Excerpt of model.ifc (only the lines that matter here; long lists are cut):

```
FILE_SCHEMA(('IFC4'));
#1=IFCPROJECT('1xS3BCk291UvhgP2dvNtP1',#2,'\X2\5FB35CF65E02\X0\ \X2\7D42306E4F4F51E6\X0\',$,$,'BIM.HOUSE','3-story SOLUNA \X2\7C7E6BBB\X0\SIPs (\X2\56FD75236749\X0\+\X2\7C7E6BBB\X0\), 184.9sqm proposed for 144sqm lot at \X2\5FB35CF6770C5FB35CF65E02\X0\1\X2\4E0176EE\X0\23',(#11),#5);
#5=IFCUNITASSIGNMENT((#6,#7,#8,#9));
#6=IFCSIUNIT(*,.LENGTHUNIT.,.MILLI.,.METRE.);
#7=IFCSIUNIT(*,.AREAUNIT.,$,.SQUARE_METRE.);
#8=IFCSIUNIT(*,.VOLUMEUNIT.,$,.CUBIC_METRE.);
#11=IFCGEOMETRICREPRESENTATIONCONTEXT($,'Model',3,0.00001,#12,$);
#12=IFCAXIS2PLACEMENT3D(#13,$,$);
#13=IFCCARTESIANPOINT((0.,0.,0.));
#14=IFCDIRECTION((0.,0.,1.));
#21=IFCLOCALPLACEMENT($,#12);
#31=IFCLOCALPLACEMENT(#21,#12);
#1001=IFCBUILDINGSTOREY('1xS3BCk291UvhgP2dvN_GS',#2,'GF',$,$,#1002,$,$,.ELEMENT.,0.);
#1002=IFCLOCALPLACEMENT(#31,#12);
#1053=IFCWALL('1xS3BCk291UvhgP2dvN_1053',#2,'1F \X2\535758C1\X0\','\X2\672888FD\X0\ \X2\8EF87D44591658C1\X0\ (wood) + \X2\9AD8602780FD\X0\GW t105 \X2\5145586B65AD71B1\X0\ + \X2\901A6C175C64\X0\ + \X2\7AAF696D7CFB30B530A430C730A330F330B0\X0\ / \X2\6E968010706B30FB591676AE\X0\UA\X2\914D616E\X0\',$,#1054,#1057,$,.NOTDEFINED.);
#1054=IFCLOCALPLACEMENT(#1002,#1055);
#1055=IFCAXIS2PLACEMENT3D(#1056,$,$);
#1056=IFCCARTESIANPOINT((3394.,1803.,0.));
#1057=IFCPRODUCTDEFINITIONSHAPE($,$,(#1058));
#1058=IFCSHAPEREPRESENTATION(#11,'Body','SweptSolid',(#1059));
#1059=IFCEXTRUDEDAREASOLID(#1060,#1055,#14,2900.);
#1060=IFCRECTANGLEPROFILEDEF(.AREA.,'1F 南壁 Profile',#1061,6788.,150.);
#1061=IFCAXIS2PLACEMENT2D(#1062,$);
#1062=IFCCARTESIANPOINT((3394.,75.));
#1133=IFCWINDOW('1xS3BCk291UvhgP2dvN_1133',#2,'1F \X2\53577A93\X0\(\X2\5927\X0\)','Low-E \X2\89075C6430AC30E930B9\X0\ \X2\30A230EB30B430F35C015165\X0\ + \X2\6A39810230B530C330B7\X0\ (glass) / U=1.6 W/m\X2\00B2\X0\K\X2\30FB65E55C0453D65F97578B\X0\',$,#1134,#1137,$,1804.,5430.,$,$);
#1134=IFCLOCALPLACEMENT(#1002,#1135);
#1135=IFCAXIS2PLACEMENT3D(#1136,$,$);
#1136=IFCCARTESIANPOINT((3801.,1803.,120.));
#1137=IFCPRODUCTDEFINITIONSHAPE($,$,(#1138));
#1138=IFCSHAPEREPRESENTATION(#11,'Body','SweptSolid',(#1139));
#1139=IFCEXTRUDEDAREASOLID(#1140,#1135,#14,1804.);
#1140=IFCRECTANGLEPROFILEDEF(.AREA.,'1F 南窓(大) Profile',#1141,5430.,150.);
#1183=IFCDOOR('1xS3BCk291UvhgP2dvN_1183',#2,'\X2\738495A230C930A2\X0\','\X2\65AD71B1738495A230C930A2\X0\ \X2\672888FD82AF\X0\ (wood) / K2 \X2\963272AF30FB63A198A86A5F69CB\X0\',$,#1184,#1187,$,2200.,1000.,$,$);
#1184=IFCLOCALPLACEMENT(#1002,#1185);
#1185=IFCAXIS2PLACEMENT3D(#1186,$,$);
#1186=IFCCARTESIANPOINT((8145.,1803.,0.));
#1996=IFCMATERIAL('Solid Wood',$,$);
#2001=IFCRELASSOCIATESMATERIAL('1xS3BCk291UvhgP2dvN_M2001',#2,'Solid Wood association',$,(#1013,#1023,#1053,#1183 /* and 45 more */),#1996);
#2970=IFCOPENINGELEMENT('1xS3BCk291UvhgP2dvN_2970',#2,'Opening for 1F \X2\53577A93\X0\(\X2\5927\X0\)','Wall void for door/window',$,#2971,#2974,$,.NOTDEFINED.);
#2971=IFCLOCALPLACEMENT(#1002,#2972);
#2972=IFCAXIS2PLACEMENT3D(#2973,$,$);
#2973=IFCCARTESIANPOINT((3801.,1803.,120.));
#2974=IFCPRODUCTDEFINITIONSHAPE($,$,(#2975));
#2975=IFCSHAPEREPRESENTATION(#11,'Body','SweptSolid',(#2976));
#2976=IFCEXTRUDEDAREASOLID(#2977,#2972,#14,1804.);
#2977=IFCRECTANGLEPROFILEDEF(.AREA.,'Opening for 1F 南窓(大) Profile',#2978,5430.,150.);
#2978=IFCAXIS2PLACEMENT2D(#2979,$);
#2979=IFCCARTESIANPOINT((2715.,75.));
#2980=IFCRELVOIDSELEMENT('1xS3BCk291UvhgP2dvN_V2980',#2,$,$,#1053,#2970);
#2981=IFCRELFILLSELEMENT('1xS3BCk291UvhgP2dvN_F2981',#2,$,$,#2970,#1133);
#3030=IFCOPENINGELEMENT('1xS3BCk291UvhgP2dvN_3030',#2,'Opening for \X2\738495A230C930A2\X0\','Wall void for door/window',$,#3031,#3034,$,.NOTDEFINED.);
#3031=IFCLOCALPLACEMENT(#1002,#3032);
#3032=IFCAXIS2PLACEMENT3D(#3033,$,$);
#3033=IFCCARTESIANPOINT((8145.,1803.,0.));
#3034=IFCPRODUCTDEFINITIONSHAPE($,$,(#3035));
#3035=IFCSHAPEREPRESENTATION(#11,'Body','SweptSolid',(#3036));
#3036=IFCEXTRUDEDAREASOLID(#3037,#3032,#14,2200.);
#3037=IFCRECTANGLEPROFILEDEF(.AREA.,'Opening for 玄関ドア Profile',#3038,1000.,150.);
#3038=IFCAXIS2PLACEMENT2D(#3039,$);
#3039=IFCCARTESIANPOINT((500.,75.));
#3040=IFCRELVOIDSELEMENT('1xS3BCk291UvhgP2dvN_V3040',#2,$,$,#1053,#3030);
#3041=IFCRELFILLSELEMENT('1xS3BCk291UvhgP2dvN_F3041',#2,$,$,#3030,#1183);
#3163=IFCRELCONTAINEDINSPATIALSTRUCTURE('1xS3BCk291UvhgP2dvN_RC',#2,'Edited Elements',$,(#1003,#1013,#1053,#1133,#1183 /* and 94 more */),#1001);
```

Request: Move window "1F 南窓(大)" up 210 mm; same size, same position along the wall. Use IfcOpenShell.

```python
import numpy as np
import ifcopenshell
import ifcopenshell.api.geometry
import ifcopenshell.util.placement
import ifcopenshell.util.unit

model = ifcopenshell.open("model.ifc")
unit_scale = ifcopenshell.util.unit.calculate_unit_scale(model)

window = model.by_guid("1xS3BCk291UvhgP2dvN_1133")
opening = window.FillsVoids[0].RelatingOpeningElement
dz = 0.21 / unit_scale

shift = np.array([0.0, 0.0, dz])
# The window is not placed relative to its opening, so move both.
for product in (opening, window):
    matrix = ifcopenshell.util.placement.get_local_placement(product.ObjectPlacement)
    matrix[:3, 3] += shift
    ifcopenshell.api.geometry.edit_object_placement(model, product=product, matrix=matrix, is_si=False)

print(f"moved by {dz * unit_scale:+.3f} m")

model.write("model_v2.ifc")
```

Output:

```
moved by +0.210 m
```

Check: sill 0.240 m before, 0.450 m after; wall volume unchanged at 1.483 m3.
